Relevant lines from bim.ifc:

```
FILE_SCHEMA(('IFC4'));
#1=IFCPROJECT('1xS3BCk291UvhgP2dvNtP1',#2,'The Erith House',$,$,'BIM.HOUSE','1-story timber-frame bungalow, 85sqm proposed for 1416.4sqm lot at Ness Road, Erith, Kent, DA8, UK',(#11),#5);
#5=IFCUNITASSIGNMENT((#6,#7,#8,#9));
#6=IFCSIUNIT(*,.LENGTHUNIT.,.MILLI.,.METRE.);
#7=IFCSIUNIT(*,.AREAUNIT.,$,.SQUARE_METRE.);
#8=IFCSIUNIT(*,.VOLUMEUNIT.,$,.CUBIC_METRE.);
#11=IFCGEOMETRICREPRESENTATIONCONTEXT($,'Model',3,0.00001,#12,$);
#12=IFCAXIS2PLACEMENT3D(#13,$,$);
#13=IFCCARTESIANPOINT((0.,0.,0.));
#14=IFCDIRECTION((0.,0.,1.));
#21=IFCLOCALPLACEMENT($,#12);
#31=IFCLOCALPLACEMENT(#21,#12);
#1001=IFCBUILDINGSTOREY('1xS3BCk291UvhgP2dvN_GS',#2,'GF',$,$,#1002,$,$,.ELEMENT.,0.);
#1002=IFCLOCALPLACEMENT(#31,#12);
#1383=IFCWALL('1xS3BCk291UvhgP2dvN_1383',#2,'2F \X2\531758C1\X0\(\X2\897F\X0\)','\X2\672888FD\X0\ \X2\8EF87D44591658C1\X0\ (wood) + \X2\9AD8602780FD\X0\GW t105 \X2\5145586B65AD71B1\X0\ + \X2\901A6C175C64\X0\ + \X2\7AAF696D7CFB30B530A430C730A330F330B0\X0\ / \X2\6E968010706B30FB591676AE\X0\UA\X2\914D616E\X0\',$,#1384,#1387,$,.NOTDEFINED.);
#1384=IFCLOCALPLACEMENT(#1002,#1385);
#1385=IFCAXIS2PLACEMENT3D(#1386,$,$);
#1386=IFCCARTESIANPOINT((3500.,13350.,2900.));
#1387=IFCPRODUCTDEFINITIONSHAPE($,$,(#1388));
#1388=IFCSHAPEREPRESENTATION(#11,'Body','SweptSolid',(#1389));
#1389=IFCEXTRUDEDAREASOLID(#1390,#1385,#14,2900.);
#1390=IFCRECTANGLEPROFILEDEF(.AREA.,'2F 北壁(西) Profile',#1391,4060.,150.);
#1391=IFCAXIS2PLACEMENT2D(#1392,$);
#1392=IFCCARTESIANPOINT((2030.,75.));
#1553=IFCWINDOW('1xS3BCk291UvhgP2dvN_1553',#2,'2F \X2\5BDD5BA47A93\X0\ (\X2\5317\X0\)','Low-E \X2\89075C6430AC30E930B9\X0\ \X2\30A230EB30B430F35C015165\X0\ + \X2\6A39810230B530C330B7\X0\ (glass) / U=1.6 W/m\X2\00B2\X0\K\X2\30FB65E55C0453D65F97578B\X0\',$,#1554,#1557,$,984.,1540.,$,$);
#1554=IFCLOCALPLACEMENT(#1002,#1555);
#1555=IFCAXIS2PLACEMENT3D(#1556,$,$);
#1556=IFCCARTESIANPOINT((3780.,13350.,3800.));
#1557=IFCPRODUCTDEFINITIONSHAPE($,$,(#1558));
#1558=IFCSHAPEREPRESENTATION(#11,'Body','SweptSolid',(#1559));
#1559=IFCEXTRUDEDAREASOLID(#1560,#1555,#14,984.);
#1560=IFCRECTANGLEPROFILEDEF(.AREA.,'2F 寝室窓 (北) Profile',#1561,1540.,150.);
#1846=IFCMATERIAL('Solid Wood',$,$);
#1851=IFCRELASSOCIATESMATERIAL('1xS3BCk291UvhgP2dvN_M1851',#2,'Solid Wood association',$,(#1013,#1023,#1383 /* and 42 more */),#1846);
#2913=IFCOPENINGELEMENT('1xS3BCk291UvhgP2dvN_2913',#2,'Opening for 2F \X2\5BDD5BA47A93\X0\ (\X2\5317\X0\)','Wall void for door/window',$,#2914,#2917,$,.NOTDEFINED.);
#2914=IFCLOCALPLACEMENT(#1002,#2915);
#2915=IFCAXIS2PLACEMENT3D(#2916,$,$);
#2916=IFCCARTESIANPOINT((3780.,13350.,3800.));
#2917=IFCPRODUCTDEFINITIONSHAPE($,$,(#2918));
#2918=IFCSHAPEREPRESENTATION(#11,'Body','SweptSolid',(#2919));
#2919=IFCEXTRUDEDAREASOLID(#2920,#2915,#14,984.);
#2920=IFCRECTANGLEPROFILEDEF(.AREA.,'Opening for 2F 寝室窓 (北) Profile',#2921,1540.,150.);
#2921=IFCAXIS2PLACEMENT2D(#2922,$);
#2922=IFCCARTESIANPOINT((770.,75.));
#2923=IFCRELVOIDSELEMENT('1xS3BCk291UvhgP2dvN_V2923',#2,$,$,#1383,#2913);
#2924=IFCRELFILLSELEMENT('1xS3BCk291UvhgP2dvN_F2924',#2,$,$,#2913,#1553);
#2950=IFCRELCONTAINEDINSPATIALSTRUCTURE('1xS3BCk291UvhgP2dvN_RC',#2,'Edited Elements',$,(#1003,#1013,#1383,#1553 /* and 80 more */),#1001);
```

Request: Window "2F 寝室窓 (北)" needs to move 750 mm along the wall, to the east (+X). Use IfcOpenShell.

```python
import ifcopenshell
import ifcopenshell.api.geometry
import ifcopenshell.util.placement

model = ifcopenshell.open("bim.ifc")

window = model.by_guid("1xS3BCk291UvhgP2dvN_1553")
opening = window.FillsVoids[0].RelatingOpeningElement
wall = opening.VoidsElements[0].RelatingBuildingElement

wall_matrix = ifcopenshell.util.placement.get_local_placement(wall.ObjectPlacement)
shift = wall_matrix[:3, 0] * 750.0
before = ifcopenshell.util.placement.get_local_placement(window.ObjectPlacement)[:3, 3].copy()

# The window is not placed relative to its opening, so move both.
for product in (opening, window):
    matrix = ifcopenshell.util.placement.get_local_placement(product.ObjectPlacement)
    matrix[:3, 3] += shift
    ifcopenshell.api.geometry.edit_object_placement(model, product=product, matrix=matrix, is_si=False)

after = ifcopenshell.util.placement.get_local_placement(window.ObjectPlacement)[:3, 3]
print("window moved by", (after - before).round(3) + 0.0)

model.write("bim_v2.ifc")
```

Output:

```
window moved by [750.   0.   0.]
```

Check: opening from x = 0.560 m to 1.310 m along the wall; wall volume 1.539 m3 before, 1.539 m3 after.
